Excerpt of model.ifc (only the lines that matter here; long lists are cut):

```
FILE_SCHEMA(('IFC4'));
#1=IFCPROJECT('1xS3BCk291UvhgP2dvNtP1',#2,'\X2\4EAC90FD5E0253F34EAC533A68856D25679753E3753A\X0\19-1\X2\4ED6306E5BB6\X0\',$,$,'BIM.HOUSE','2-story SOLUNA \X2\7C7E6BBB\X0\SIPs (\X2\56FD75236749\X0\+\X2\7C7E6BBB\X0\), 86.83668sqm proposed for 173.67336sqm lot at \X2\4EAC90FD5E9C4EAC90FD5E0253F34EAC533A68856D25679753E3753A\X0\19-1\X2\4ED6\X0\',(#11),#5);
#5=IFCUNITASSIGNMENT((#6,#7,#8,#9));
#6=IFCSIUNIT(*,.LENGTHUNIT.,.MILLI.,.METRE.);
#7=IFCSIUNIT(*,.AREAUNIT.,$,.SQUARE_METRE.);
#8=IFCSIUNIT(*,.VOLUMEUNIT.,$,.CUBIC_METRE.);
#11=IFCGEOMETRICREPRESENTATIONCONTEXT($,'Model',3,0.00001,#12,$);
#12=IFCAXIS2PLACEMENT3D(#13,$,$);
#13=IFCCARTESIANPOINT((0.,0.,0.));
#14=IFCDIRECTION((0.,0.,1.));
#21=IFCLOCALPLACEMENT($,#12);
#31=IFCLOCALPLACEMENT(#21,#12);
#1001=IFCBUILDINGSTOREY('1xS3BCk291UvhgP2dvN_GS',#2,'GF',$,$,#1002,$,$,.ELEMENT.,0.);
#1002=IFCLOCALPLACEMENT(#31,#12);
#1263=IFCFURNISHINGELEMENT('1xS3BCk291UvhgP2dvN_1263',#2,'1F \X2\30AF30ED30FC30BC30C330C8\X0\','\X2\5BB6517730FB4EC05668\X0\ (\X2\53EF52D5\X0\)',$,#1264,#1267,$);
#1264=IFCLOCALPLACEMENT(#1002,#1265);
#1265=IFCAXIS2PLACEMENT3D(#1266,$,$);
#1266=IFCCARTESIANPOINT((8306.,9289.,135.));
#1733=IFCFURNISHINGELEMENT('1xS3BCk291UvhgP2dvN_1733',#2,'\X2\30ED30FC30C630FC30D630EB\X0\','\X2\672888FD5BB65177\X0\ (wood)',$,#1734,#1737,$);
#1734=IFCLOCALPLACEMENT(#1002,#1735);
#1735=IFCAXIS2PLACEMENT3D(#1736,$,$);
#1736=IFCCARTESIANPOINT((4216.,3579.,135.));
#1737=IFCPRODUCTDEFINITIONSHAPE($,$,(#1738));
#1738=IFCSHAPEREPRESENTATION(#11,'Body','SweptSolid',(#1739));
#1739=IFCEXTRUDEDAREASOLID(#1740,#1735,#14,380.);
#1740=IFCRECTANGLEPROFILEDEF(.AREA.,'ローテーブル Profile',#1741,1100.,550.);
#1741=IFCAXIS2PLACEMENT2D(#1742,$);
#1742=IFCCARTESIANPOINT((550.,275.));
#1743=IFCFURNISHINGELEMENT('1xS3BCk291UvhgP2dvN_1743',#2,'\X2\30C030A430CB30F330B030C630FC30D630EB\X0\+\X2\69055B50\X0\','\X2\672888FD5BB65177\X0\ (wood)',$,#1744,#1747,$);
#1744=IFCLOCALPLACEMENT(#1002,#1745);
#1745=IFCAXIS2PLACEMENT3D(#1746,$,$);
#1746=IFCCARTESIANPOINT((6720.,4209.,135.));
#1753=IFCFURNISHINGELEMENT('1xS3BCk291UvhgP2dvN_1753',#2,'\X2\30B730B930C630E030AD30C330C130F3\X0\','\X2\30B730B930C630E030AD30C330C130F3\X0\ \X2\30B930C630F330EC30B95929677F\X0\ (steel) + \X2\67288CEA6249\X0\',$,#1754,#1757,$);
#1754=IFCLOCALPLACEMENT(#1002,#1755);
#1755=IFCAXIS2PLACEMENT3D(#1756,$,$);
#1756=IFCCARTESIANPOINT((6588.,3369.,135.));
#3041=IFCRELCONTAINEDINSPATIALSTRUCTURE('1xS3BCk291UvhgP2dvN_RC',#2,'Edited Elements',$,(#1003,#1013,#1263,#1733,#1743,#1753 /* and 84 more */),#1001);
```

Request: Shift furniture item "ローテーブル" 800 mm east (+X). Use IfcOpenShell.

```python
import ifcopenshell
import ifcopenshell.api.geometry
import ifcopenshell.util.placement

model = ifcopenshell.open("model.ifc")

item = model.by_guid("1xS3BCk291UvhgP2dvN_1733")
matrix = ifcopenshell.util.placement.get_local_placement(item.ObjectPlacement)
matrix[0, 3] += 800.0
ifcopenshell.api.geometry.edit_object_placement(model, product=item, matrix=matrix, is_si=False)

print(ifcopenshell.util.placement.get_local_placement(item.ObjectPlacement).round(3) + 0.0)

model.write("model-out.ifc")
```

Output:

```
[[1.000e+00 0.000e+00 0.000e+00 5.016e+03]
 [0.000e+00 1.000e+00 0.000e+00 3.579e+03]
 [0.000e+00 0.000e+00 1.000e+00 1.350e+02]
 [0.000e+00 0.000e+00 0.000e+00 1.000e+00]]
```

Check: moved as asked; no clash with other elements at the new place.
